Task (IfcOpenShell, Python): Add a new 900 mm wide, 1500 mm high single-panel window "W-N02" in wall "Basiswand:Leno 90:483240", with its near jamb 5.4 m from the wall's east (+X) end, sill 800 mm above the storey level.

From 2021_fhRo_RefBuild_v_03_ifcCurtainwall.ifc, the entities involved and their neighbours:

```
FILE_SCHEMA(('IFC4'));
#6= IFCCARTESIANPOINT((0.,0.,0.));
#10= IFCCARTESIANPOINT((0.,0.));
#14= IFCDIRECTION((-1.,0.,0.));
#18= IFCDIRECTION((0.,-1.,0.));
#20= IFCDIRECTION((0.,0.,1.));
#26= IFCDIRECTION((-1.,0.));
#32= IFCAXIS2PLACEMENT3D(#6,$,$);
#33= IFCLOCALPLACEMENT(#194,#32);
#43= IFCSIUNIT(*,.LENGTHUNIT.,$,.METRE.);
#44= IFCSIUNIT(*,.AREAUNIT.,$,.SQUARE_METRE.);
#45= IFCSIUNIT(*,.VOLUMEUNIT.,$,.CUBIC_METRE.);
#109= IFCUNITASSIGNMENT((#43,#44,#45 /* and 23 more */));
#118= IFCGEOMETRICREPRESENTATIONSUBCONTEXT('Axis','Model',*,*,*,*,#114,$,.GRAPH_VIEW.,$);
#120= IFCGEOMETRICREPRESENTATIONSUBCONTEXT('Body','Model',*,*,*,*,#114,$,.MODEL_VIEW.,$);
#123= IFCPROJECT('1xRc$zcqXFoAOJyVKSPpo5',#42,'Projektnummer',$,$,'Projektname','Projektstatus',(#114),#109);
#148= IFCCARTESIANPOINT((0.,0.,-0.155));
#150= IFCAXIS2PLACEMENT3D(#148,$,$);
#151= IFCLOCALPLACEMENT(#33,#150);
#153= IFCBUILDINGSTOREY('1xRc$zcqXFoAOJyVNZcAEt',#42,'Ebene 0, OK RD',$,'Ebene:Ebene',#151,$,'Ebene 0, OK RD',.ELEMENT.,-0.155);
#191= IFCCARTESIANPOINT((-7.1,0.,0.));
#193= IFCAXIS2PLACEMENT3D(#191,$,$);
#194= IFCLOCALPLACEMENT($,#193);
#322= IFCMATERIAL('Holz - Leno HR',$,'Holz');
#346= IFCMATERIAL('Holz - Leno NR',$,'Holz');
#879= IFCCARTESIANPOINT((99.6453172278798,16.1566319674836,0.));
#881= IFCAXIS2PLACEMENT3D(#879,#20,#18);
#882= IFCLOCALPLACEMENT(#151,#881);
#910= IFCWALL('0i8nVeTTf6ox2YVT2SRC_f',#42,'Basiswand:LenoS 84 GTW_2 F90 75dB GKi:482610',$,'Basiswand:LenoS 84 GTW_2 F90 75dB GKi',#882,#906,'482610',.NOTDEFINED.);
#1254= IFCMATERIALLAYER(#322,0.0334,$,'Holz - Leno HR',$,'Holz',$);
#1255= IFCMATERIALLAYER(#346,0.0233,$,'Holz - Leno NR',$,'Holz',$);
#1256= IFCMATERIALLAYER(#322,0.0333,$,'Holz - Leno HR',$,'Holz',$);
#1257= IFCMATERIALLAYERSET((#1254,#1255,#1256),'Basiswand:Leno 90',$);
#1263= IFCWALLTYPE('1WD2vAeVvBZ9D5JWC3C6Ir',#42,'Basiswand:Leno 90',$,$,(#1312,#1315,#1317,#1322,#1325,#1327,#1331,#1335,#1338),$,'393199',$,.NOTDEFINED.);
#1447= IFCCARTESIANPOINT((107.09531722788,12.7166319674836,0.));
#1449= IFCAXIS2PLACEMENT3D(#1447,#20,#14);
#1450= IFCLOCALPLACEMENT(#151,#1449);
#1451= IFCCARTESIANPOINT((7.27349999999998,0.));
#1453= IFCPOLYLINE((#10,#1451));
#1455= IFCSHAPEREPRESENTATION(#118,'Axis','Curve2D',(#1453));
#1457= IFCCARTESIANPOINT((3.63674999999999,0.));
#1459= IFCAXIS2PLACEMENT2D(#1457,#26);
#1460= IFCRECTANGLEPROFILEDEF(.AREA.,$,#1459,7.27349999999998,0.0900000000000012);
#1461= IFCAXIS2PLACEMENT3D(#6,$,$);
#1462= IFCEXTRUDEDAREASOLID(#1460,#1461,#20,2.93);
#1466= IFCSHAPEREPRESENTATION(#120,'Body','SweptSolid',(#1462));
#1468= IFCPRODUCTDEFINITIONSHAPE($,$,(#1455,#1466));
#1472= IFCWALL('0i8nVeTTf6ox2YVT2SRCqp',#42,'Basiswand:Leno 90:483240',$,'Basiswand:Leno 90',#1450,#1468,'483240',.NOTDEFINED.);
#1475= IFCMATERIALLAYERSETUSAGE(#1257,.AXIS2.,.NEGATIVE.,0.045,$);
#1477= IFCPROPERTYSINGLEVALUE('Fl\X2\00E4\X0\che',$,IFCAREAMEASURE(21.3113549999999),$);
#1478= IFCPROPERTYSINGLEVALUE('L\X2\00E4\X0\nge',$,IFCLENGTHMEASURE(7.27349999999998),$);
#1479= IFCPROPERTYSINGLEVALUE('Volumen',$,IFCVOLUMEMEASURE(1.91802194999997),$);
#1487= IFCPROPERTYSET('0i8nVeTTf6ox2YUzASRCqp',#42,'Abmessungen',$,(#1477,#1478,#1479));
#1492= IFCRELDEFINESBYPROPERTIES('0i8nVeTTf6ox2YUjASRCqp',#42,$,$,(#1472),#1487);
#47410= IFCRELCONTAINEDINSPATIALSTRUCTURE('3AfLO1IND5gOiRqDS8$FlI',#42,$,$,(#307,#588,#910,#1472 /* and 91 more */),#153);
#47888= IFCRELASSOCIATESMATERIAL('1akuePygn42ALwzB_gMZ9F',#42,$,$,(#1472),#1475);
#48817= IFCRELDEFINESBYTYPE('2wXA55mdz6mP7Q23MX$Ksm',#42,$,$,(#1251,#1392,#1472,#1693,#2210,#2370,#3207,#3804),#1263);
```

```python
import numpy as np
import ifcopenshell
import ifcopenshell.api.feature
import ifcopenshell.api.geometry
import ifcopenshell.api.pset
import ifcopenshell.api.root
import ifcopenshell.api.spatial
import ifcopenshell.geom
import ifcopenshell.util.element
import ifcopenshell.util.placement
import ifcopenshell.util.representation
import ifcopenshell.util.shape
import ifcopenshell.util.unit

model = ifcopenshell.open("2021_fhRo_RefBuild_v_03_ifcCurtainwall.ifc")
unit_scale = ifcopenshell.util.unit.calculate_unit_scale(model)
area_scale = ifcopenshell.util.unit.calculate_unit_scale(model, "AREAUNIT")
volume_scale = ifcopenshell.util.unit.calculate_unit_scale(model, "VOLUMEUNIT")
settings = ifcopenshell.geom.settings()


def volume(element):
    """Net volume in cubic metres, openings subtracted."""
    shape = ifcopenshell.geom.create_shape(settings, element)
    return ifcopenshell.util.shape.get_volume(shape.geometry)


wall = model.by_id(1472)
storey = ifcopenshell.util.element.get_container(wall, ifc_class="IfcBuildingStorey")
context = ifcopenshell.util.representation.get_context(model, "Model", "Body", "MODEL_VIEW")
before = volume(wall)

width, height, from_end, sill = 0.9, 1.5, 5.4, 0.8  # metres

# The wall runs along its own X axis, and the end named is its -X end.
wall_shape = ifcopenshell.geom.create_shape(settings, wall)
x, y, z = ifcopenshell.util.shape.get_vertices(wall_shape.geometry).T
start = x.min() + from_end
face, thickness = float(y.min()), float(y.max() - y.min())
wall_matrix = ifcopenshell.util.placement.get_local_placement(wall.ObjectPlacement)
level = ifcopenshell.util.placement.get_local_placement(storey.ObjectPlacement)[2, 3]


def in_wall(x, y):
    """Placement at x, y metres in the wall's axes, at sill height."""
    matrix = wall_matrix.copy()
    matrix[:, 3] = wall_matrix @ np.array([x / unit_scale, y / unit_scale, 0.0, 1.0])
    matrix[2, 3] = level + sill / unit_scale
    return matrix


# Opening: a box that overshoots both wall faces by 50 mm.
opening = ifcopenshell.api.root.create_entity(model, ifc_class="IfcOpeningElement", predefined_type="OPENING")
box = ifcopenshell.api.geometry.add_wall_representation(
    model, context=context, length=width, height=height, thickness=thickness + 0.1
)
ifcopenshell.api.geometry.assign_representation(model, product=opening, representation=box)
ifcopenshell.api.geometry.edit_object_placement(model, product=opening, matrix=in_wall(start, face - 0.05), is_si=False)
ifcopenshell.api.feature.add_feature(model, feature=opening, element=wall)

window = ifcopenshell.api.root.create_entity(model, ifc_class="IfcWindow", name="W-N02", predefined_type="WINDOW")
window.OverallWidth, window.OverallHeight = width / unit_scale, height / unit_scale
window.PartitioningType = "SINGLE_PANEL"
body = ifcopenshell.api.geometry.add_window_representation(
    model,
    context=context,
    overall_width=window.OverallWidth,
    overall_height=window.OverallHeight,
    partition_type="SINGLE_PANEL",
)
ifcopenshell.api.geometry.assign_representation(model, product=window, representation=body)
ifcopenshell.api.spatial.assign_container(model, products=[window], relating_structure=storey)
ifcopenshell.api.feature.add_filling(model, opening=opening, element=window)

# Centre the window in the wall's thickness.
ifcopenshell.api.geometry.edit_object_placement(model, product=window, matrix=in_wall(start, face), is_si=False)
window_shape = ifcopenshell.geom.create_shape(settings, window)
depth = ifcopenshell.util.shape.get_vertices(window_shape.geometry)[:, 1]
offset = face + thickness / 2 - (depth.min() + depth.max()) / 2
ifcopenshell.api.geometry.edit_object_placement(model, product=window, matrix=in_wall(start, offset), is_si=False)

after = volume(wall)

# Update the wall's stored quantities.
pset = model.by_id(ifcopenshell.util.element.get_pset(wall, "Abmessungen", should_inherit=False)["id"])
ifcopenshell.api.pset.edit_pset(model, pset=pset, properties={
    "Fläche": model.create_entity("IfcAreaMeasure", after / thickness / area_scale),
    "Volumen": model.create_entity("IfcVolumeMeasure", after / volume_scale),
})

print(f"wall volume {before:.3f} -> {after:.3f} m3")

model.write("2021_fhRo_RefBuild_v_03_ifcCurtainwall_rev.ifc")
```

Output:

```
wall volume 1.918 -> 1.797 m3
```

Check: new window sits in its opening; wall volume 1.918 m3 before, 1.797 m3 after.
